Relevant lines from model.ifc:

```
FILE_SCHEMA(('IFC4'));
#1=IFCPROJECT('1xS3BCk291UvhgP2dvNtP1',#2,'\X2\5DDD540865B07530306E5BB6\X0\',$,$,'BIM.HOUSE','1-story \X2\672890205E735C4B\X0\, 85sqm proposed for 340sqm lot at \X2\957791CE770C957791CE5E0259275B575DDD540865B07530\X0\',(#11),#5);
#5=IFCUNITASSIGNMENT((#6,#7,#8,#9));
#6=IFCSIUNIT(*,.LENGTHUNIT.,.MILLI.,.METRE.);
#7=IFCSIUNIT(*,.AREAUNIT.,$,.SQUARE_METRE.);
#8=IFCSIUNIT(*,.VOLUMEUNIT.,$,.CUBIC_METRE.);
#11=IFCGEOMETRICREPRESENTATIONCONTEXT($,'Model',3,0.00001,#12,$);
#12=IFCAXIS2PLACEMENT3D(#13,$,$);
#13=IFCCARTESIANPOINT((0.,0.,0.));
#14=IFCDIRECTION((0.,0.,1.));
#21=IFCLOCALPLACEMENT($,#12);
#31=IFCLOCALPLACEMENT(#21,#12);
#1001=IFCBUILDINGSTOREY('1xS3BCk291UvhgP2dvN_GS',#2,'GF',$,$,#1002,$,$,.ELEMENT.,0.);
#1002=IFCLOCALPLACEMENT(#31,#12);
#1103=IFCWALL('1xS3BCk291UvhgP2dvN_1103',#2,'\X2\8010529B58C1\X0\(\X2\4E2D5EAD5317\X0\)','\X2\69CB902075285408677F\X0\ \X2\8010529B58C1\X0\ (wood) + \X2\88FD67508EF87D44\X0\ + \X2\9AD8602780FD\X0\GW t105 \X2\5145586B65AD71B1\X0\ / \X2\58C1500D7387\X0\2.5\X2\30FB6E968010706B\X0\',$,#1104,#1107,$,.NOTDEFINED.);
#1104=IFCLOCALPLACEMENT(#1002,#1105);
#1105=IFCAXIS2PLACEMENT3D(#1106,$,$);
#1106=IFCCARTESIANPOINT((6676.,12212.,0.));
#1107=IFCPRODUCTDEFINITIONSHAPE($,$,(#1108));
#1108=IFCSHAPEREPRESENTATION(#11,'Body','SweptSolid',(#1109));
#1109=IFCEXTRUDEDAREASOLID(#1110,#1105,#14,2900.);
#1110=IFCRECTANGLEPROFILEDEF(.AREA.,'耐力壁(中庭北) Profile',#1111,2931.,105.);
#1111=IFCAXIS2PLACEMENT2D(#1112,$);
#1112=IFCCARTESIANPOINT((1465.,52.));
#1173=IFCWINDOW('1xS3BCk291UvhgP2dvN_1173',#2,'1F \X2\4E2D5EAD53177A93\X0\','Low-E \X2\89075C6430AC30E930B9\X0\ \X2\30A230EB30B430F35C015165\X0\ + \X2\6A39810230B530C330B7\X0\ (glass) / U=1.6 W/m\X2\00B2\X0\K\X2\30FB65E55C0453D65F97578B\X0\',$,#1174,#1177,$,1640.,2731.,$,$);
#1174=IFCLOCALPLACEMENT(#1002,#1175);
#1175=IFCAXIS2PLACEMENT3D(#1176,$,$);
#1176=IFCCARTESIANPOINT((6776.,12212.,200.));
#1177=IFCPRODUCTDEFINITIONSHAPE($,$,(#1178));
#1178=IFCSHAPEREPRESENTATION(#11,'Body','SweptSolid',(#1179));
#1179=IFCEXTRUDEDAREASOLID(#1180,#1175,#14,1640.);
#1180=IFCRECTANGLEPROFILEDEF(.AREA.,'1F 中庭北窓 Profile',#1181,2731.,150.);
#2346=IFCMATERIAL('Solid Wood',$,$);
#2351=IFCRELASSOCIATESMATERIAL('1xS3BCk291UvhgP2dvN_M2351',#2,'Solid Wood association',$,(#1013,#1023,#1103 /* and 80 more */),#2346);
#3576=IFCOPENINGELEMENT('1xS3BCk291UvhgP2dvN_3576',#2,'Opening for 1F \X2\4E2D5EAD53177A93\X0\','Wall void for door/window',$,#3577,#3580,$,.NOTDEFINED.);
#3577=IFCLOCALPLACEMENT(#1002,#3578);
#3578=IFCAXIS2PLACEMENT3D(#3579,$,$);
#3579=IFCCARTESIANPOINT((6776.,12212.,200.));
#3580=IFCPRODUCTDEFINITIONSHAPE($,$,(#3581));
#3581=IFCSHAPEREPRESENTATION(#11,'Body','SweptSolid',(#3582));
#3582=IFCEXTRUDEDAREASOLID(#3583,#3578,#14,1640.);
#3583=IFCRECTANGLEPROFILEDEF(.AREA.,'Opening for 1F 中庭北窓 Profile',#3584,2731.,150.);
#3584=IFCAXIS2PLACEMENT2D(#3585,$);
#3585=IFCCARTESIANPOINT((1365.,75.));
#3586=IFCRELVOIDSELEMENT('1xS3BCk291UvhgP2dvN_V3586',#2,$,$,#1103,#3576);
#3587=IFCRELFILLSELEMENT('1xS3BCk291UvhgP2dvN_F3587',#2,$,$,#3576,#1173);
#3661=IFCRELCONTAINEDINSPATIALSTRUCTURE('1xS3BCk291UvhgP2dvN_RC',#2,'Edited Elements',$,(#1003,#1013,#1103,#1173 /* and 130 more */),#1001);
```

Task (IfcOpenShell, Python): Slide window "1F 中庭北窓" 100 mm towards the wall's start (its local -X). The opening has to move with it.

```python
import ifcopenshell
import ifcopenshell.api.geometry
import ifcopenshell.util.placement
import ifcopenshell.util.unit

model = ifcopenshell.open("model.ifc")
unit_scale = ifcopenshell.util.unit.calculate_unit_scale(model)

window = model.by_guid("1xS3BCk291UvhgP2dvN_1173")
opening = window.FillsVoids[0].RelatingOpeningElement
wall = opening.VoidsElements[0].RelatingBuildingElement

wall_matrix = ifcopenshell.util.placement.get_local_placement(wall.ObjectPlacement)
shift = wall_matrix[:3, 0] * -0.1 / unit_scale
before = ifcopenshell.util.placement.get_local_placement(window.ObjectPlacement)[:3, 3].copy()

# The window is not placed relative to its opening, so move both.
for product in (opening, window):
    matrix = ifcopenshell.util.placement.get_local_placement(product.ObjectPlacement)
    matrix[:3, 3] += shift
    ifcopenshell.api.geometry.edit_object_placement(model, product=product, matrix=matrix, is_si=False)

after = ifcopenshell.util.placement.get_local_placement(window.ObjectPlacement)[:3, 3]
print("window moved by", (after - before).round(3) + 0.0)

model.write("model_edited.ifc")
```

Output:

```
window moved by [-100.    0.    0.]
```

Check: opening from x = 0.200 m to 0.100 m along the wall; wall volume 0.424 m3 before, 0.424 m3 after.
